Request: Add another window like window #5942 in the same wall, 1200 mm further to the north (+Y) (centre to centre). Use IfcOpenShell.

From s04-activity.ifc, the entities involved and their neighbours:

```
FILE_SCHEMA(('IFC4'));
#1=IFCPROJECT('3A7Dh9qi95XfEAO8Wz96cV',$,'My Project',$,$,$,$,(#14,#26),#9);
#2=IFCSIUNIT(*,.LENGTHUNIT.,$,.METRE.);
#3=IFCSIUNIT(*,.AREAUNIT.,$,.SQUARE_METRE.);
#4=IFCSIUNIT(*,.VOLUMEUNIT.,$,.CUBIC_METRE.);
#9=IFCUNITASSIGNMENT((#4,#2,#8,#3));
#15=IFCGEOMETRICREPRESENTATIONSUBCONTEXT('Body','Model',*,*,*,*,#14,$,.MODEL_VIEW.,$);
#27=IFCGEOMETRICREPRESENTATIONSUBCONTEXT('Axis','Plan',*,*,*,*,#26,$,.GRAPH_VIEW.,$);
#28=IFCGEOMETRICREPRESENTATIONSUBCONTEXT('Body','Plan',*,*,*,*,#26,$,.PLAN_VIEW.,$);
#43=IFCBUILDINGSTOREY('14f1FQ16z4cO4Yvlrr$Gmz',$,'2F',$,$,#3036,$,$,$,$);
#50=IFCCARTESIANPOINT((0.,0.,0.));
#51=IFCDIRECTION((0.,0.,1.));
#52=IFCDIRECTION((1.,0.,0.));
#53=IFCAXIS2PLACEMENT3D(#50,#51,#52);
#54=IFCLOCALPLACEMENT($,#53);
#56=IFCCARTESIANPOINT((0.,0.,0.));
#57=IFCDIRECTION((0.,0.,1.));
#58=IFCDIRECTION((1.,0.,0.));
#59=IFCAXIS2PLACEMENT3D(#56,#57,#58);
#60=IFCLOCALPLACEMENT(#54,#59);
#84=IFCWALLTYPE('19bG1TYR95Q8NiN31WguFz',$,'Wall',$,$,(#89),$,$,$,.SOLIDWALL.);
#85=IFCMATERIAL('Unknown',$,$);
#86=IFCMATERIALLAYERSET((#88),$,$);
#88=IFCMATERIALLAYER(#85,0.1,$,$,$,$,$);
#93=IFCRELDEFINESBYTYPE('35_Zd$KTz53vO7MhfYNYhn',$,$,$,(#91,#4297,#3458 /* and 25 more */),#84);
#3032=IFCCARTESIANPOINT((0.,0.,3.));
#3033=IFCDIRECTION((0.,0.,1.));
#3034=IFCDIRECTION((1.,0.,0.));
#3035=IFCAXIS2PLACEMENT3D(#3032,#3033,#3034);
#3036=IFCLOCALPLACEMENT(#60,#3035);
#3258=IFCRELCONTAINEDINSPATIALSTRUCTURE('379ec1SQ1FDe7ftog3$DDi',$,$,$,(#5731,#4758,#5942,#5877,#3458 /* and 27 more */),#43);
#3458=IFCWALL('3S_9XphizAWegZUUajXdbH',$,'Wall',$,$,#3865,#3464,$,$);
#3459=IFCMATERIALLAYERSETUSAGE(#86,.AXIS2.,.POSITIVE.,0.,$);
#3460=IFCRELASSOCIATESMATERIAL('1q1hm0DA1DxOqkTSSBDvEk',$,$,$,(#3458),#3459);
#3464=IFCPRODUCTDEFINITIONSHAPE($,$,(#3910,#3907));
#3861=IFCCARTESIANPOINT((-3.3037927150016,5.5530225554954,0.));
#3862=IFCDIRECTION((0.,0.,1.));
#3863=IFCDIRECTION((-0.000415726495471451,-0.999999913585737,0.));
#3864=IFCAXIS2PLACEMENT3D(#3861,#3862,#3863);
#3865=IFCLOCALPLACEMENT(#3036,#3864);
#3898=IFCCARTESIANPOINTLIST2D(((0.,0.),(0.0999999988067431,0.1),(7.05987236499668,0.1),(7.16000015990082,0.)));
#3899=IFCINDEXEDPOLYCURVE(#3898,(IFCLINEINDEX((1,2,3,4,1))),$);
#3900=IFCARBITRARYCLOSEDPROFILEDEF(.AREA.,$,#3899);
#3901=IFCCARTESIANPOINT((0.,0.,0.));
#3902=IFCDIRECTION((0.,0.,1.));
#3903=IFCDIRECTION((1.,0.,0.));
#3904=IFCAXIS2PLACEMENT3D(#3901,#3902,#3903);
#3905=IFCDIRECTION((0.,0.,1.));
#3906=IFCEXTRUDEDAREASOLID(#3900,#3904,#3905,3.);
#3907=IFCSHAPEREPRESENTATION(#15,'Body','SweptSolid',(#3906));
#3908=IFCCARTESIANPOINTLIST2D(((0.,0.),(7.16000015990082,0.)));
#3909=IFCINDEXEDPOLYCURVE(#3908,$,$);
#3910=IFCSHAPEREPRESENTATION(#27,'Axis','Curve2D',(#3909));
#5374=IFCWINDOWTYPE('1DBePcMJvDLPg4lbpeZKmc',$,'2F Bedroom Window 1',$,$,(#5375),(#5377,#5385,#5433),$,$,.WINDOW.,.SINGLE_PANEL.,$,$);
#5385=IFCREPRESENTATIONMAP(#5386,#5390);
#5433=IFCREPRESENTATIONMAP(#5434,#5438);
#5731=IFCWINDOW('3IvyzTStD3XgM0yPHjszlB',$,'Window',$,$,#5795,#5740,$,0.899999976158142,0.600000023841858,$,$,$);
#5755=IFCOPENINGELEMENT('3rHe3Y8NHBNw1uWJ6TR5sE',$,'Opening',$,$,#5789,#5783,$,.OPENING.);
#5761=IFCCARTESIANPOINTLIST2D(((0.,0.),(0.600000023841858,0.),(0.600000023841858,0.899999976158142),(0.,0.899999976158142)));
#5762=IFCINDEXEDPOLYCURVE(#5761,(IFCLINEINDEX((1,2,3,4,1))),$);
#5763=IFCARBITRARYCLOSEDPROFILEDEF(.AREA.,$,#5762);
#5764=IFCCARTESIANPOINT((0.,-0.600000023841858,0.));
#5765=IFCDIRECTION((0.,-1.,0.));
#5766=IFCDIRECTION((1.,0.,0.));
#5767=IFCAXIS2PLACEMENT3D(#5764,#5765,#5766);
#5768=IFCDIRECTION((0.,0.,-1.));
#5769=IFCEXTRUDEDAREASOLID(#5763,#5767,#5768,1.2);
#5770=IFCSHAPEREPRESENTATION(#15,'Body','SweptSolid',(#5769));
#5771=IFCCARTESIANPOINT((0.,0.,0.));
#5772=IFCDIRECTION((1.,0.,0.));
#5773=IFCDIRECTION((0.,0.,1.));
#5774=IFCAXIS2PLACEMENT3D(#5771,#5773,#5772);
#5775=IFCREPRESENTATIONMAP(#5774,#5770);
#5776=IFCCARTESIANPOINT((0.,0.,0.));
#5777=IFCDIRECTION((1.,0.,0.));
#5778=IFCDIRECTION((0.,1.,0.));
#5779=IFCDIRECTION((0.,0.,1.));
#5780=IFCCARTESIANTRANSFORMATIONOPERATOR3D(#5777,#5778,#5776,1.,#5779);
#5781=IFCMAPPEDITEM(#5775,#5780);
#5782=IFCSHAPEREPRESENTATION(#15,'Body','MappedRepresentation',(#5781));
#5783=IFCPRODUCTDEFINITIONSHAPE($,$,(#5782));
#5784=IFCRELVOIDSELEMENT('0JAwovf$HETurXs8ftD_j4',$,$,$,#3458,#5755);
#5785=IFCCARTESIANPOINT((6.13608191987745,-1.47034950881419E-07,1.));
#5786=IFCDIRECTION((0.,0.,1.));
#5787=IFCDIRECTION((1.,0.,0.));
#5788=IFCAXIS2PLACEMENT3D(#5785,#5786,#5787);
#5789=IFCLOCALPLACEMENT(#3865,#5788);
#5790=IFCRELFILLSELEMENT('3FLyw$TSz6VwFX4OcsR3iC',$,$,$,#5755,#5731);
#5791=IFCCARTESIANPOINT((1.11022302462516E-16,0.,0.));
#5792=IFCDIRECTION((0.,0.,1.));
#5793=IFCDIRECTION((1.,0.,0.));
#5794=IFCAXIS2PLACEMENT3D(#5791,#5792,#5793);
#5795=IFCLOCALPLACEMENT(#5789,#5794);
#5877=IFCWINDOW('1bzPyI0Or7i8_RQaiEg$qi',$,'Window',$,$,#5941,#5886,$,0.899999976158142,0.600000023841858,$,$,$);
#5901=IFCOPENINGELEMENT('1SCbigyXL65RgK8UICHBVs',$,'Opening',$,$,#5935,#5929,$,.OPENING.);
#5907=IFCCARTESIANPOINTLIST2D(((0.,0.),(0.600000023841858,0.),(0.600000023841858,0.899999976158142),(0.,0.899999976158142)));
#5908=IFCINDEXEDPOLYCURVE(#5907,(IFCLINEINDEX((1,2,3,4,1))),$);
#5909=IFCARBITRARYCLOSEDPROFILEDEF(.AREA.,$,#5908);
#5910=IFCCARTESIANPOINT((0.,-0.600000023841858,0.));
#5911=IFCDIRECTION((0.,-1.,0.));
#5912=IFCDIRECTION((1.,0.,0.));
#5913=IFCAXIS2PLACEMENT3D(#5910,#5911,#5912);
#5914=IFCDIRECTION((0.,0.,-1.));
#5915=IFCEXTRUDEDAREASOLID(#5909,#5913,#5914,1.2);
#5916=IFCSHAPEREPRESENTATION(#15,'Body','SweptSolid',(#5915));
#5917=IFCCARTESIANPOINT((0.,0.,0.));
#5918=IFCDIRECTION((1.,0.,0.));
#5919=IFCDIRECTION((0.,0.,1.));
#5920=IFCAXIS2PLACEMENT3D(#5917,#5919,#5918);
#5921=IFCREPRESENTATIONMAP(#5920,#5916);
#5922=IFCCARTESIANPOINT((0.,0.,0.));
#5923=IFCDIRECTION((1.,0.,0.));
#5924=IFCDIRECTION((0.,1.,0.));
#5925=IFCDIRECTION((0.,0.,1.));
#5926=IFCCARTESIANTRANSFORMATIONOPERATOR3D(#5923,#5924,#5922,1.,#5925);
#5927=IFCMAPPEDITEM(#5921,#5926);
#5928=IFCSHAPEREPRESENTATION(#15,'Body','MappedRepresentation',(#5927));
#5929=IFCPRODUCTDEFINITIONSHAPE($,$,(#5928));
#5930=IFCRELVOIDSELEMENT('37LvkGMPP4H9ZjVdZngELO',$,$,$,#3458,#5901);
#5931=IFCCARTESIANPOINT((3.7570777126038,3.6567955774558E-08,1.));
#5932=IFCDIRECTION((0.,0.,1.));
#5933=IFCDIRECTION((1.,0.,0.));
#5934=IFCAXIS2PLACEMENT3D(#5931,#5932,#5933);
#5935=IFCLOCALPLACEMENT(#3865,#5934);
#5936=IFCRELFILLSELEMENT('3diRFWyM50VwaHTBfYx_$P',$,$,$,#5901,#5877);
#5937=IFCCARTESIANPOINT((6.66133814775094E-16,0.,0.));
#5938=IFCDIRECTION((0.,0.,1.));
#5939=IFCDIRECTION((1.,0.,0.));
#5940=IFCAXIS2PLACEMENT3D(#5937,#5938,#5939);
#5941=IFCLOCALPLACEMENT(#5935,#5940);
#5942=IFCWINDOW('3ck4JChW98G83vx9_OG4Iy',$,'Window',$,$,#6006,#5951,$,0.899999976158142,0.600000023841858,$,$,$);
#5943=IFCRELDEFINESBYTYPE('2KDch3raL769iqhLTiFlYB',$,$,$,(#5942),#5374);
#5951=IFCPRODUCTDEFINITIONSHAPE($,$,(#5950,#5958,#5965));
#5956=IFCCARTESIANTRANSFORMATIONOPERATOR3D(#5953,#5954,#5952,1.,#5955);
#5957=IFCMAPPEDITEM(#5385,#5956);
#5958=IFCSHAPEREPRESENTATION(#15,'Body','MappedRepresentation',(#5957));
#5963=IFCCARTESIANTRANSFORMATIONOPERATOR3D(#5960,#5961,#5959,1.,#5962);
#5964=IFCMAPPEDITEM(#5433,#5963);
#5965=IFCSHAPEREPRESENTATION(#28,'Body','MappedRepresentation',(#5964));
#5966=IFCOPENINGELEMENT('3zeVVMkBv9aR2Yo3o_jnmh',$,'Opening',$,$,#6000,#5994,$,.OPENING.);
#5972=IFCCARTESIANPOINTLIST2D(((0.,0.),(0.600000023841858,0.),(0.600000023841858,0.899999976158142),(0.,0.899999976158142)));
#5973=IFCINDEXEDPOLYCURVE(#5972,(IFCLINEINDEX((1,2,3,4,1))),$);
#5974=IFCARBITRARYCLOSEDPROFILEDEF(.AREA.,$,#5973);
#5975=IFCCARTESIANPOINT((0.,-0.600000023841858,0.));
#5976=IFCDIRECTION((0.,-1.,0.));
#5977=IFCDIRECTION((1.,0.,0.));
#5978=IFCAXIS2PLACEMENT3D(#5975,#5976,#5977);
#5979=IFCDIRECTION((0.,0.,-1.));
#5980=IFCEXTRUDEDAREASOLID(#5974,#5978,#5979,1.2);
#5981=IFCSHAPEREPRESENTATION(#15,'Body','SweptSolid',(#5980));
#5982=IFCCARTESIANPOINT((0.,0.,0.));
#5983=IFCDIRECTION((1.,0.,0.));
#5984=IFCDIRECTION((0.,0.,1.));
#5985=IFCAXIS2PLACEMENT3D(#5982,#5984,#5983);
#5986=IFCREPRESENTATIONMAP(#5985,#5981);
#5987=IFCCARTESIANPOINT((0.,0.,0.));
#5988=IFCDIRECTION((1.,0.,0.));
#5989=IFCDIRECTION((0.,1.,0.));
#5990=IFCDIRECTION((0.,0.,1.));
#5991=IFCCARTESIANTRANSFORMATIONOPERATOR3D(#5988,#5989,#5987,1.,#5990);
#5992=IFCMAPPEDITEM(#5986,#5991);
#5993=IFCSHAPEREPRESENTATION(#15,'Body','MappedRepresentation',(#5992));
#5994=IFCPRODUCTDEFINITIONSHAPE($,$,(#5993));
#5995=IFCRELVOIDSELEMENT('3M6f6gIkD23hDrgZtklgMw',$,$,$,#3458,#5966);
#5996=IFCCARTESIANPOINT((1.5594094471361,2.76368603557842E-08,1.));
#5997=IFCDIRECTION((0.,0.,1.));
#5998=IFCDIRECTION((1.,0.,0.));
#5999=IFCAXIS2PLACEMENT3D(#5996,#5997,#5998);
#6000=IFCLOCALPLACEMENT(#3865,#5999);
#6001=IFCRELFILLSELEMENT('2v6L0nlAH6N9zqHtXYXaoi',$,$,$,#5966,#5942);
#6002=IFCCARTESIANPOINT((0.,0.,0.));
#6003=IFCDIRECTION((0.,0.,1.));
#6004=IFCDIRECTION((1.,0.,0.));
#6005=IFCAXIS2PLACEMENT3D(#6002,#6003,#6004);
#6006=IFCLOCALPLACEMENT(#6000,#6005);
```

```python
import ifcopenshell
import ifcopenshell.api.feature
import ifcopenshell.api.geometry
import ifcopenshell.api.root
import ifcopenshell.geom
import ifcopenshell.util.element
import ifcopenshell.util.placement
import ifcopenshell.util.shape

model = ifcopenshell.open("s04-activity.ifc")
settings = ifcopenshell.geom.settings()


def volume(element):
    """Net volume in cubic metres, openings subtracted."""
    shape = ifcopenshell.geom.create_shape(settings, element)
    return ifcopenshell.util.shape.get_volume(shape.geometry)


window = model.by_id(5942)
opening = window.FillsVoids[0].RelatingOpeningElement
wall = opening.VoidsElements[0].RelatingBuildingElement
before = volume(wall)
shift = ifcopenshell.util.placement.get_local_placement(wall.ObjectPlacement)[:3, 0] * -1.2

# copy_class copies the void relationship, type, container and properties, but no geometry.
new_opening = ifcopenshell.api.root.copy_class(model, product=opening)
new_opening.Representation = ifcopenshell.util.element.copy_deep(
    model, opening.Representation, exclude=["IfcGeometricRepresentationContext", "IfcRepresentationMap"]
)
new_window = ifcopenshell.api.root.copy_class(model, product=window)
new_window.Representation = ifcopenshell.util.element.copy_deep(
    model, window.Representation, exclude=["IfcGeometricRepresentationContext", "IfcRepresentationMap"]
)
ifcopenshell.api.feature.add_filling(model, opening=new_opening, element=new_window)

for old, new in ((opening, new_opening), (window, new_window)):
    matrix = ifcopenshell.util.placement.get_local_placement(old.ObjectPlacement)
    matrix[:3, 3] += shift
    ifcopenshell.api.geometry.edit_object_placement(model, product=new, matrix=matrix, is_si=False)

after = volume(wall)

print(f"wall volume {before:.3f} -> {after:.3f} m3")

model.write("s04-activity_edited.ifc")
```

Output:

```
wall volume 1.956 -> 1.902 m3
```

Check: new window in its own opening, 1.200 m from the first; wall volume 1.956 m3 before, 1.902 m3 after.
